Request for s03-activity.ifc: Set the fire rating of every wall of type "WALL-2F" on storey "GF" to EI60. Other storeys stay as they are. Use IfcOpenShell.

First a look at what the model holds.

```python
import ifcopenshell
import ifcopenshell.util.element

model = ifcopenshell.open("s03-activity.ifc")
print(model.schema)
storey = next(s for s in model.by_type("IfcBuildingStorey") if s.Name == "GF")
walls = [e for e in ifcopenshell.util.element.get_decomposition(storey) if e.is_a("IfcWall")]
seen = {}
for e in walls:
    element_type = ifcopenshell.util.element.get_type(e)
    key = (element_type.Name if element_type != e and element_type else None, ifcopenshell.util.element.get_pset(e, "Pset_WallCommon", "FireRating"))
    seen[key] = seen.get(key, 0) + 1
for (name, value), count in sorted(seen.items(), key=str):
    print(count, "x", name, "|", value)
```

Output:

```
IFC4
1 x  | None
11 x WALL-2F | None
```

```python
import ifcopenshell
import ifcopenshell.api.pset
import ifcopenshell.util.element

model = ifcopenshell.open("s03-activity.ifc")

storey = next(s for s in model.by_type("IfcBuildingStorey") if s.Name == "GF")
walls = [e for e in ifcopenshell.util.element.get_decomposition(storey) if e.is_a("IfcWall")]

count = 0
for e in walls:
    element_type = ifcopenshell.util.element.get_type(e)
    if element_type in (None, e) or element_type.Name != "WALL-2F":
        continue
    # add_pset returns the element's existing set when there is one.
    pset = ifcopenshell.api.pset.add_pset(model, product=e, name="Pset_WallCommon")
    ifcopenshell.api.pset.edit_pset(model, pset=pset, properties={"FireRating": "EI60"})
    count += 1

print(count, "walls updated")

model.write("s03-activity_rev.ifc")
```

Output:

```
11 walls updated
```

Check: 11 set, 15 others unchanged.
